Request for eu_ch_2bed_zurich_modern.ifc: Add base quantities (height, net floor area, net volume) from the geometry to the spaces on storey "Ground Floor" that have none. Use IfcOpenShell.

First a look at what the model holds.

```python
import ifcopenshell
import ifcopenshell.util.element
import ifcopenshell.util.unit

model = ifcopenshell.open("eu_ch_2bed_zurich_modern.ifc")
print(model.schema)
for unit_type in ("LENGTHUNIT", "AREAUNIT", "VOLUMEUNIT"):
    print(unit_type, ifcopenshell.util.unit.calculate_unit_scale(model, unit_type))
storey = next(s for s in model.by_type("IfcBuildingStorey") if s.Name == "Ground Floor")
spaces = [e for e in ifcopenshell.util.element.get_decomposition(storey) if e.is_a("IfcSpace")]
for e in sorted(spaces, key=lambda e: e.id()):
    print(e.id(), e.is_a(), e.Name, list(ifcopenshell.util.element.get_psets(e, qtos_only=True)), sep=" | ")
```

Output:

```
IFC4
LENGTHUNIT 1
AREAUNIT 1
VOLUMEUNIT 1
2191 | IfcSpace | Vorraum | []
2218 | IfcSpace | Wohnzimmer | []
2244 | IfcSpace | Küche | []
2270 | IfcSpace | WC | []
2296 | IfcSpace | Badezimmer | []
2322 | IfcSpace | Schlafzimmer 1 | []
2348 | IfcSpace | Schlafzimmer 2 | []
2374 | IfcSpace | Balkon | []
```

```python
import ifcopenshell
import ifcopenshell.api.pset
import ifcopenshell.geom
import ifcopenshell.util.element
import ifcopenshell.util.shape
import ifcopenshell.util.unit

model = ifcopenshell.open("eu_ch_2bed_zurich_modern.ifc")
unit_scale = ifcopenshell.util.unit.calculate_unit_scale(model)
area_scale = ifcopenshell.util.unit.calculate_unit_scale(model, "AREAUNIT")
volume_scale = ifcopenshell.util.unit.calculate_unit_scale(model, "VOLUMEUNIT")
settings = ifcopenshell.geom.settings()

storey = next(s for s in model.by_type("IfcBuildingStorey") if s.Name == "Ground Floor")
spaces = [e for e in ifcopenshell.util.element.get_decomposition(storey) if e.is_a("IfcSpace")]

for e in sorted(spaces, key=lambda e: e.id()):
    if ifcopenshell.util.element.get_psets(e, qtos_only=True, should_inherit=False):
        continue
    # Geometry comes back in metres, in the element's own axes.
    shape = ifcopenshell.geom.create_shape(settings, e)
    values = {
        "Height": ifcopenshell.util.shape.get_z(shape.geometry) / unit_scale,
        "NetFloorArea": ifcopenshell.util.shape.get_footprint_area(shape.geometry) / area_scale,
        "NetVolume": ifcopenshell.util.shape.get_volume(shape.geometry) / volume_scale,
    }
    qto = ifcopenshell.api.pset.add_qto(model, product=e, name="Qto_SpaceBaseQuantities")
    ifcopenshell.api.pset.edit_qto(model, qto=qto, properties=values)
    print(e.id(), {k: round(v, 3) for k, v in values.items()})

model.write("eu_ch_2bed_zurich_modern_edited.ifc")
```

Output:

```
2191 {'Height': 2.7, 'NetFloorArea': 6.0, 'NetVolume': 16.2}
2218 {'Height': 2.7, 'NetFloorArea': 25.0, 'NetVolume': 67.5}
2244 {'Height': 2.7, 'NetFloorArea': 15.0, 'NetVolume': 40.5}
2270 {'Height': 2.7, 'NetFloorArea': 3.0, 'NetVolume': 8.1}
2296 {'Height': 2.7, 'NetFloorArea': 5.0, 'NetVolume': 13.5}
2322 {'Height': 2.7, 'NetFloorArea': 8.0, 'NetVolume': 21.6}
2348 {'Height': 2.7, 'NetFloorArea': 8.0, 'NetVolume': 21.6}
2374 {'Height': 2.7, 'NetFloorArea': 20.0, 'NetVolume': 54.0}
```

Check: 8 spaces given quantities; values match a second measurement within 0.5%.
